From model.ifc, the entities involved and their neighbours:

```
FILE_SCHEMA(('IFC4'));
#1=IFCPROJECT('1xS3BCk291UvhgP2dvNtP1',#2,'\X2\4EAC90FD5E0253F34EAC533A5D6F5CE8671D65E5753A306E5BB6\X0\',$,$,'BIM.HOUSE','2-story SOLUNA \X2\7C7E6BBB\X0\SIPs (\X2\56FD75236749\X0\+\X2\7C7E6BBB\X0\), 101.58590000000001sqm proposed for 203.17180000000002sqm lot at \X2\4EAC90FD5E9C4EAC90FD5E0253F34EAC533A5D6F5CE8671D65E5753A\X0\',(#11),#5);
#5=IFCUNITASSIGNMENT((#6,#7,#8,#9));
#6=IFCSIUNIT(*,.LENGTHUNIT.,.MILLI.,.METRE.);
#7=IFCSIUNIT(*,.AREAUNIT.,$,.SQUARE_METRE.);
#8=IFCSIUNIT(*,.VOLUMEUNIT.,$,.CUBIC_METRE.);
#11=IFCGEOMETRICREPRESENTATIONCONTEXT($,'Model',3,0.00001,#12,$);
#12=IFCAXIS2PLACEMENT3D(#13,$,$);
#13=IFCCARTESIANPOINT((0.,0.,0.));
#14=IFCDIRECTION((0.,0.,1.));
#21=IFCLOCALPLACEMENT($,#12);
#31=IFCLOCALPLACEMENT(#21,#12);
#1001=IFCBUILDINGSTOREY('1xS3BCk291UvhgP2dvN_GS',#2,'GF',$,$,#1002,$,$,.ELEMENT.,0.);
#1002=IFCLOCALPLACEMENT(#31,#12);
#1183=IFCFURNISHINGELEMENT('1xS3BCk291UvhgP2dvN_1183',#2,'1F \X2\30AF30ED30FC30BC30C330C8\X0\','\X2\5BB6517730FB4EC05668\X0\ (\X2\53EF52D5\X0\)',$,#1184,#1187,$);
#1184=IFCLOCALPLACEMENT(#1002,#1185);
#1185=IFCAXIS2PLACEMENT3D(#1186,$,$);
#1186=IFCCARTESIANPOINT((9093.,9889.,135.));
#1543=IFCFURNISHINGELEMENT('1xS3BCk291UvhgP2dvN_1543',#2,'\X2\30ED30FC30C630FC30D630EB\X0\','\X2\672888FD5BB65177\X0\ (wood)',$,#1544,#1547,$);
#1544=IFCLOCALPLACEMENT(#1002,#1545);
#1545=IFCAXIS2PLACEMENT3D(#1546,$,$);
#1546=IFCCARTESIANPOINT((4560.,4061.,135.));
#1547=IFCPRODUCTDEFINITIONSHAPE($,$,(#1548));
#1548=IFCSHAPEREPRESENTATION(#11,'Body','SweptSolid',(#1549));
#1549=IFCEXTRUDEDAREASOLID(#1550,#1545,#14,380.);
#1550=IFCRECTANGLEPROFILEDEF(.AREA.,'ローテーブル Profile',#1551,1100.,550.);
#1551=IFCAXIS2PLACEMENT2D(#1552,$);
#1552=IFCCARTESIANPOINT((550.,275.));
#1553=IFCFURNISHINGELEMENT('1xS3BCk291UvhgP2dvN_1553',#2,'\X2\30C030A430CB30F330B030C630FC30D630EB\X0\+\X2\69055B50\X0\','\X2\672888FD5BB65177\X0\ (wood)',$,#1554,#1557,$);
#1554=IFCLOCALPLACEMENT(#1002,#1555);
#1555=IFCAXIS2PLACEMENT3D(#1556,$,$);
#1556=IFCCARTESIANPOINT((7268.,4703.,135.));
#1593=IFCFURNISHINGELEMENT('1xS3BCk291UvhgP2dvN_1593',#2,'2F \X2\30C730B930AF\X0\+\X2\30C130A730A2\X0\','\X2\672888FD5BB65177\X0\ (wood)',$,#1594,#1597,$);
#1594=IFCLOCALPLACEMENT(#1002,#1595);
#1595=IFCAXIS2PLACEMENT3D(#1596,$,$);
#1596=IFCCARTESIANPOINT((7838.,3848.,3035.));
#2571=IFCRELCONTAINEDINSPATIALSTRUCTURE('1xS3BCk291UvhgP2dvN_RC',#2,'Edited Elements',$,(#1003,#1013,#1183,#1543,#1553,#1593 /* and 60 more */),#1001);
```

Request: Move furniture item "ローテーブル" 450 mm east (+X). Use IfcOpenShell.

```python
import ifcopenshell
import ifcopenshell.api.geometry
import ifcopenshell.util.placement
import ifcopenshell.util.unit

model = ifcopenshell.open("model.ifc")
unit_scale = ifcopenshell.util.unit.calculate_unit_scale(model)

item = model.by_guid("1xS3BCk291UvhgP2dvN_1543")
matrix = ifcopenshell.util.placement.get_local_placement(item.ObjectPlacement)
matrix[0, 3] += 0.45 / unit_scale
ifcopenshell.api.geometry.edit_object_placement(model, product=item, matrix=matrix, is_si=False)

print(ifcopenshell.util.placement.get_local_placement(item.ObjectPlacement).round(3) + 0.0)

model.write("model_v2.ifc")
```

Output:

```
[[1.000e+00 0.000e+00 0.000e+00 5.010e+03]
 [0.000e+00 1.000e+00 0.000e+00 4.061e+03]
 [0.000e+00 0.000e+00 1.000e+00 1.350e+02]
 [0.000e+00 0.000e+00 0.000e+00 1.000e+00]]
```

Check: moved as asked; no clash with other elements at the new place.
